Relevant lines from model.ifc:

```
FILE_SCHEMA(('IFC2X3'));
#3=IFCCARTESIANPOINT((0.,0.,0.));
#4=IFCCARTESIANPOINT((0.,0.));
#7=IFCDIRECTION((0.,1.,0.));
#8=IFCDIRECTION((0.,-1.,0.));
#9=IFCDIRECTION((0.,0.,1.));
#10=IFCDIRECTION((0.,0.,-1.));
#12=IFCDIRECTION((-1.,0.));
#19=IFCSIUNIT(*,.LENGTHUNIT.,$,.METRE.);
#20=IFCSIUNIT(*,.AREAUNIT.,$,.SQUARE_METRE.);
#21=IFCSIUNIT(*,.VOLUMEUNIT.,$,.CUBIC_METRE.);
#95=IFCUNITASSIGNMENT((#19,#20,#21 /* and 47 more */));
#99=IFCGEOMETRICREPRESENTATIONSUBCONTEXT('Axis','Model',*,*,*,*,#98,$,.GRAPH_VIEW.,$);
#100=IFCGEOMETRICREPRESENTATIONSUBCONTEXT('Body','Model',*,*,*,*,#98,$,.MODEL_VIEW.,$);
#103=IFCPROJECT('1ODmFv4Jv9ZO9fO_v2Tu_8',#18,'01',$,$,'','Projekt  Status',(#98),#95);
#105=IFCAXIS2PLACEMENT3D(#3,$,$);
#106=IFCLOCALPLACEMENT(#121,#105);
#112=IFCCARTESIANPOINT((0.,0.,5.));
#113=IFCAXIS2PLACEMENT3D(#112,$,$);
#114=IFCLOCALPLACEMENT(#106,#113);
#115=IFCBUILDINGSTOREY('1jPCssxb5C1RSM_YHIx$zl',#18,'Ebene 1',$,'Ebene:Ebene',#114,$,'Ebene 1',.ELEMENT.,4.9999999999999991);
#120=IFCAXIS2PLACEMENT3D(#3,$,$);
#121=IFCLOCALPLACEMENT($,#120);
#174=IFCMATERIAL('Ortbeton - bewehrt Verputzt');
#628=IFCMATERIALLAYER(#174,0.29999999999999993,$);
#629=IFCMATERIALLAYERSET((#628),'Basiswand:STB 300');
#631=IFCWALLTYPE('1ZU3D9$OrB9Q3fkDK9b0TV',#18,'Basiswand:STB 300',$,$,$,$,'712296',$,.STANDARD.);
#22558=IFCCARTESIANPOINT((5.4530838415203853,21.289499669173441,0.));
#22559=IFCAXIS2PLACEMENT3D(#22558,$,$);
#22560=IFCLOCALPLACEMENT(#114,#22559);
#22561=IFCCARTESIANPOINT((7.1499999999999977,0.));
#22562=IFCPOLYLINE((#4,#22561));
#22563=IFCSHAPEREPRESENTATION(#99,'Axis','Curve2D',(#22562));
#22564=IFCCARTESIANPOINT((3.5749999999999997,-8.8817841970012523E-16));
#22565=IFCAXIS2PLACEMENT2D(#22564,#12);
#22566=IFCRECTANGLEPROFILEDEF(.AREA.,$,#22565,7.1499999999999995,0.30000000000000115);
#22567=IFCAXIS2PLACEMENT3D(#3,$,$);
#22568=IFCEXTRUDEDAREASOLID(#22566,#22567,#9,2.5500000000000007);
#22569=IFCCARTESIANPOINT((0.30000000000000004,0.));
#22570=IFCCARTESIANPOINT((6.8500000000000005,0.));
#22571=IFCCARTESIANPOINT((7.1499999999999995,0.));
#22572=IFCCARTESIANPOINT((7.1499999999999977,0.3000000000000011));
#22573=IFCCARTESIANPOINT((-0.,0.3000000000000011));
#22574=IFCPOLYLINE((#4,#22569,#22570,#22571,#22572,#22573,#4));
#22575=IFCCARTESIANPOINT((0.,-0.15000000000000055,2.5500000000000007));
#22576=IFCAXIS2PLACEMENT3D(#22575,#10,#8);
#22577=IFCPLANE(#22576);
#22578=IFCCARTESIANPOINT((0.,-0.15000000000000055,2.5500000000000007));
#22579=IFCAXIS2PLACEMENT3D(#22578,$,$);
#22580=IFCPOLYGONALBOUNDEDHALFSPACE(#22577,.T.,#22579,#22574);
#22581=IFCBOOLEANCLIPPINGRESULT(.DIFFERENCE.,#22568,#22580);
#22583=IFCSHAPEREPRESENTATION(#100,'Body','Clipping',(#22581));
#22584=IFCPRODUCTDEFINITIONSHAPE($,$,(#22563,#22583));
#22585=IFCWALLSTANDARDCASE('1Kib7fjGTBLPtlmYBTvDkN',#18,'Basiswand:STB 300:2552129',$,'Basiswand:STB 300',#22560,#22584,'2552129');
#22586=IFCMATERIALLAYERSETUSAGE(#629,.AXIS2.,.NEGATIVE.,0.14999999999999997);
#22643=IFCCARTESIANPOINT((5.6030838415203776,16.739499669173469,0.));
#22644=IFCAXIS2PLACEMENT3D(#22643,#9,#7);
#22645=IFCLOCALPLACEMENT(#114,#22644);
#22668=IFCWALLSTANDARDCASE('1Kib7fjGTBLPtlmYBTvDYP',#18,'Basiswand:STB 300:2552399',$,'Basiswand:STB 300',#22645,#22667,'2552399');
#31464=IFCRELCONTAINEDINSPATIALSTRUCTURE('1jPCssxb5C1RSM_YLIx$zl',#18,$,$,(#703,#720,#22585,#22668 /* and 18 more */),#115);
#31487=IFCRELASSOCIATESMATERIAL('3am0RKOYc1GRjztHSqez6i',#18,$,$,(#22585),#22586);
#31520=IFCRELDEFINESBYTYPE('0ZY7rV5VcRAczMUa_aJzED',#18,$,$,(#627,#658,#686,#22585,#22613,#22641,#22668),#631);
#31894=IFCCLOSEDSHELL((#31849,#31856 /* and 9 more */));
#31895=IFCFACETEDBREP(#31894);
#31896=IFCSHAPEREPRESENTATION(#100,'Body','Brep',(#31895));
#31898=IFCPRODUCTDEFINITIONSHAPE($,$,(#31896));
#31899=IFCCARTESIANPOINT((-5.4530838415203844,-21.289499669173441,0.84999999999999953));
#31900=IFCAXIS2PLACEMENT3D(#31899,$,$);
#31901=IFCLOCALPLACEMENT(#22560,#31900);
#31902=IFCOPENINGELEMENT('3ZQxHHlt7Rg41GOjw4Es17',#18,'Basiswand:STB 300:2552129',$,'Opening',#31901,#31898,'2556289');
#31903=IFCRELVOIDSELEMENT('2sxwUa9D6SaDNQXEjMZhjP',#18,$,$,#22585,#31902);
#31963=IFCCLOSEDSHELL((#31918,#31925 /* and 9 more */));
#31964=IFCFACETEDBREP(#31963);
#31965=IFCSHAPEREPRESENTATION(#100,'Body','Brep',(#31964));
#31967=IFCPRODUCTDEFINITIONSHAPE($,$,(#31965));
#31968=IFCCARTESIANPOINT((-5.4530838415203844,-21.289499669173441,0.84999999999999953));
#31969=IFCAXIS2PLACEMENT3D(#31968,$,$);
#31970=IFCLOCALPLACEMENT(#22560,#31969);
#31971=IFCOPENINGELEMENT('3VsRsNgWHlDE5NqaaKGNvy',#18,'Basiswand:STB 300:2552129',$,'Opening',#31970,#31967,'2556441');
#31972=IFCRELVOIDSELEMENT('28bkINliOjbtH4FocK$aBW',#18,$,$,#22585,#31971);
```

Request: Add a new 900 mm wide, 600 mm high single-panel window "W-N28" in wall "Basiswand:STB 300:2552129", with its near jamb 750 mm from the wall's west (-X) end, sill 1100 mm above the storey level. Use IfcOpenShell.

```python
import numpy as np
import ifcopenshell
import ifcopenshell.api.feature
import ifcopenshell.api.geometry
import ifcopenshell.api.root
import ifcopenshell.api.spatial
import ifcopenshell.api.type
import ifcopenshell.geom
import ifcopenshell.util.element
import ifcopenshell.util.placement
import ifcopenshell.util.representation
import ifcopenshell.util.shape
import ifcopenshell.util.unit

model = ifcopenshell.open("model.ifc")
unit_scale = ifcopenshell.util.unit.calculate_unit_scale(model)
settings = ifcopenshell.geom.settings()


def volume(element):
    """Net volume in cubic metres, openings subtracted."""
    shape = ifcopenshell.geom.create_shape(settings, element)
    return ifcopenshell.util.shape.get_volume(shape.geometry)


wall = model.by_guid("1Kib7fjGTBLPtlmYBTvDkN")
storey = ifcopenshell.util.element.get_container(wall, ifc_class="IfcBuildingStorey")
context = ifcopenshell.util.representation.get_context(model, "Model", "Body", "MODEL_VIEW")
before = volume(wall)

width, height, from_end, sill = 0.9, 0.6, 0.75, 1.1  # metres

# The wall runs along its own X axis, and the end named is its -X end.
wall_shape = ifcopenshell.geom.create_shape(settings, wall)
x, y, z = ifcopenshell.util.shape.get_vertices(wall_shape.geometry).T
start = x.min() + from_end
face, thickness = float(y.min()), float(y.max() - y.min())
wall_matrix = ifcopenshell.util.placement.get_local_placement(wall.ObjectPlacement)
level = ifcopenshell.util.placement.get_local_placement(storey.ObjectPlacement)[2, 3]


def in_wall(x, y):
    """Placement at x, y metres in the wall's axes, at sill height."""
    matrix = wall_matrix.copy()
    matrix[:, 3] = wall_matrix @ np.array([x / unit_scale, y / unit_scale, 0.0, 1.0])
    matrix[2, 3] = level + sill / unit_scale
    return matrix


# Opening: a box that overshoots both wall faces by 50 mm.
opening = ifcopenshell.api.root.create_entity(model, ifc_class="IfcOpeningElement")
box = ifcopenshell.api.geometry.add_wall_representation(
    model, context=context, length=width, height=height, thickness=thickness + 0.1
)
ifcopenshell.api.geometry.assign_representation(model, product=opening, representation=box)
ifcopenshell.api.geometry.edit_object_placement(model, product=opening, matrix=in_wall(start, face - 0.05), is_si=False)
ifcopenshell.api.feature.add_feature(model, feature=opening, element=wall)

window = ifcopenshell.api.root.create_entity(model, ifc_class="IfcWindow", name="W-N28")
window.OverallWidth, window.OverallHeight = width / unit_scale, height / unit_scale
body = ifcopenshell.api.geometry.add_window_representation(
    model,
    context=context,
    overall_width=window.OverallWidth,
    overall_height=window.OverallHeight,
    partition_type="SINGLE_PANEL",
)
ifcopenshell.api.geometry.assign_representation(model, product=window, representation=body)
ifcopenshell.api.spatial.assign_container(model, products=[window], relating_structure=storey)
fills = ifcopenshell.api.feature.add_filling(model, opening=opening, element=window)
fills.OwnerHistory = window.OwnerHistory  # required in IFC2X3

# IFC2X3 keeps the operation on the window style.
style = ifcopenshell.api.root.create_entity(model, ifc_class="IfcWindowStyle", name="W-N28")
style.OperationType, style.ConstructionType = "SINGLE_PANEL", "NOTDEFINED"
style.ParameterTakesPrecedence = style.Sizeable = False
ifcopenshell.api.type.assign_type(model, related_objects=[window], relating_type=style)

# Centre the window in the wall's thickness.
ifcopenshell.api.geometry.edit_object_placement(model, product=window, matrix=in_wall(start, face), is_si=False)
window_shape = ifcopenshell.geom.create_shape(settings, window)
depth = ifcopenshell.util.shape.get_vertices(window_shape.geometry)[:, 1]
offset = face + thickness / 2 - (depth.min() + depth.max()) / 2
ifcopenshell.api.geometry.edit_object_placement(model, product=window, matrix=in_wall(start, offset), is_si=False)

after = volume(wall)

print(f"wall volume {before:.3f} -> {after:.3f} m3")

model.write("model_edited.ifc")
```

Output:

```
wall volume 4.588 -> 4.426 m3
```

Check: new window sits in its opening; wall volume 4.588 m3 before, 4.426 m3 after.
